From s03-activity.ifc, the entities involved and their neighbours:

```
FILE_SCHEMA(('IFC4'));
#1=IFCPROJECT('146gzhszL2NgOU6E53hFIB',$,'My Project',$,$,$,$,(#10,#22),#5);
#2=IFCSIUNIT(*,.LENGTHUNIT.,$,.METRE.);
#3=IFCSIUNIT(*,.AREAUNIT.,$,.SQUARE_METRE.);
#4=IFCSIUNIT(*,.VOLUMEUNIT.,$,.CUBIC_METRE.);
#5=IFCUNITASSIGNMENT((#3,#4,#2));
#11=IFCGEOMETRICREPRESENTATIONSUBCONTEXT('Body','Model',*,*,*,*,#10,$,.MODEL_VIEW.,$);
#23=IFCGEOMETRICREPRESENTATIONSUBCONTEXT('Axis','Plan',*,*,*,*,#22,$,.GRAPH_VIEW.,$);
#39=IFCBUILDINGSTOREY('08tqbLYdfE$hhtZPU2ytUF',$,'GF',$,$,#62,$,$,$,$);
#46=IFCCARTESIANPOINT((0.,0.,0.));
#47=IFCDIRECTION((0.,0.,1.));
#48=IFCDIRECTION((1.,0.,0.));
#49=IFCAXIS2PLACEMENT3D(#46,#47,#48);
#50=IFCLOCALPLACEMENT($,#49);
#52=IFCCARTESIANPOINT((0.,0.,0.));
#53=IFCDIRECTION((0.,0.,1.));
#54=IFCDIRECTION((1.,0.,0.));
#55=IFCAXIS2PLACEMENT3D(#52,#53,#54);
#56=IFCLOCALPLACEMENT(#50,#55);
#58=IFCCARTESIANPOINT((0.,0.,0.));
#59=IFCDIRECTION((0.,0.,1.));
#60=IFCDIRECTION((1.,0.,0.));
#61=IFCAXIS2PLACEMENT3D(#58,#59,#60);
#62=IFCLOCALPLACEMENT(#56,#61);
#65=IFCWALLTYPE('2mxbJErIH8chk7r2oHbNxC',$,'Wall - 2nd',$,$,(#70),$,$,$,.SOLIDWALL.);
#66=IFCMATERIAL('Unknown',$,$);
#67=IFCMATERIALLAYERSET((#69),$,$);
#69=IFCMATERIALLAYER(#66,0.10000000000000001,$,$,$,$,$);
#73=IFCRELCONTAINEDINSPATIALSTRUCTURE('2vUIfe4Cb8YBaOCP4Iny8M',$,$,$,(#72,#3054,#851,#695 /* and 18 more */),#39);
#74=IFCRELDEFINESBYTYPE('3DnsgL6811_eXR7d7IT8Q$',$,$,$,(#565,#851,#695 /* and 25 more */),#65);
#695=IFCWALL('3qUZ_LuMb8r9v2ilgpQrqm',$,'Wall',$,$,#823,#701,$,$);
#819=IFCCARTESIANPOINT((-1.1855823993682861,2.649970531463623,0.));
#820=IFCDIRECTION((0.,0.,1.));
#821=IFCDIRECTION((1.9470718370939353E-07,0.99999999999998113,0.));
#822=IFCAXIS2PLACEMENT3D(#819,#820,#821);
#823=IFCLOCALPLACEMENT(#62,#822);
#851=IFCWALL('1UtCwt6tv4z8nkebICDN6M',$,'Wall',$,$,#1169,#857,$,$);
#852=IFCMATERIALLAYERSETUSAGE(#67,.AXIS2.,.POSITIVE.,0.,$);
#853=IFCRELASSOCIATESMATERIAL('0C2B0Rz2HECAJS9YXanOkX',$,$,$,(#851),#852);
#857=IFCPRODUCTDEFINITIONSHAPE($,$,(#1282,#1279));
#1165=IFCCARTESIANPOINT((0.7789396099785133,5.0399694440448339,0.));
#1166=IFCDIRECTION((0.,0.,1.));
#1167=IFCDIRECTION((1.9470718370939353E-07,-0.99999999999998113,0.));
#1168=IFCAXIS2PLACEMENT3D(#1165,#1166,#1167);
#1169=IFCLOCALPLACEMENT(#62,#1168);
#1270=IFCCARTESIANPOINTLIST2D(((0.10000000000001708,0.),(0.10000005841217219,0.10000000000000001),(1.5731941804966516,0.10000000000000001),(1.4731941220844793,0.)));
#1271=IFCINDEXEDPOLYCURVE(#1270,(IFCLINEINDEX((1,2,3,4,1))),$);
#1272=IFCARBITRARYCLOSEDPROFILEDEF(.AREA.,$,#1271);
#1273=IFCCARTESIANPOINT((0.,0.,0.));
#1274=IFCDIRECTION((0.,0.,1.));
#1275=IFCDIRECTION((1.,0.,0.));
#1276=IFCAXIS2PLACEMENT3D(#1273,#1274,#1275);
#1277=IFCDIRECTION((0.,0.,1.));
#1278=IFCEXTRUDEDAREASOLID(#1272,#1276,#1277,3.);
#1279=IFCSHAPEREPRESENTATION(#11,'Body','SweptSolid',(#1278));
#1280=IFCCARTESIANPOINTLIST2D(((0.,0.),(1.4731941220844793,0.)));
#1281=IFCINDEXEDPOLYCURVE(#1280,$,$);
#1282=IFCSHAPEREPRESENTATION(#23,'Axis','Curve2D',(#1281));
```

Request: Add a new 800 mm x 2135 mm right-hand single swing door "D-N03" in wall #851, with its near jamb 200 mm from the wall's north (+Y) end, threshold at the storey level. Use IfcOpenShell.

```python
import numpy as np
import ifcopenshell
import ifcopenshell.api.feature
import ifcopenshell.api.geometry
import ifcopenshell.api.root
import ifcopenshell.api.spatial
import ifcopenshell.geom
import ifcopenshell.util.element
import ifcopenshell.util.placement
import ifcopenshell.util.representation
import ifcopenshell.util.shape
import ifcopenshell.util.unit

model = ifcopenshell.open("s03-activity.ifc")
unit_scale = ifcopenshell.util.unit.calculate_unit_scale(model)
settings = ifcopenshell.geom.settings()


def volume(element):
    """Net volume in cubic metres, openings subtracted."""
    shape = ifcopenshell.geom.create_shape(settings, element)
    return ifcopenshell.util.shape.get_volume(shape.geometry)


wall = model.by_guid("1UtCwt6tv4z8nkebICDN6M")
storey = ifcopenshell.util.element.get_container(wall, ifc_class="IfcBuildingStorey")
context = ifcopenshell.util.representation.get_context(model, "Model", "Body", "MODEL_VIEW")
before = volume(wall)

width, height, from_end, sill = 0.8, 2.135, 0.2, 0.0  # metres

# The wall runs along its own X axis, and the end named is its -X end.
wall_shape = ifcopenshell.geom.create_shape(settings, wall)
x, y, z = ifcopenshell.util.shape.get_vertices(wall_shape.geometry).T
start = x.min() + from_end
face, thickness = float(y.min()), float(y.max() - y.min())
wall_matrix = ifcopenshell.util.placement.get_local_placement(wall.ObjectPlacement)
level = ifcopenshell.util.placement.get_local_placement(storey.ObjectPlacement)[2, 3]


def in_wall(x, y):
    """Placement at x, y metres in the wall's axes, at sill height."""
    matrix = wall_matrix.copy()
    matrix[:, 3] = wall_matrix @ np.array([x / unit_scale, y / unit_scale, 0.0, 1.0])
    matrix[2, 3] = level + sill / unit_scale
    return matrix


# Opening: a box that overshoots both wall faces by 50 mm.
opening = ifcopenshell.api.root.create_entity(model, ifc_class="IfcOpeningElement", predefined_type="OPENING")
box = ifcopenshell.api.geometry.add_wall_representation(
    model, context=context, length=width, height=height, thickness=thickness + 0.1
)
ifcopenshell.api.geometry.assign_representation(model, product=opening, representation=box)
ifcopenshell.api.geometry.edit_object_placement(model, product=opening, matrix=in_wall(start, face - 0.05), is_si=False)
ifcopenshell.api.feature.add_feature(model, feature=opening, element=wall)

door = ifcopenshell.api.root.create_entity(model, ifc_class="IfcDoor", name="D-N03", predefined_type="DOOR")
door.OverallWidth, door.OverallHeight = width / unit_scale, height / unit_scale
door.OperationType = "SINGLE_SWING_RIGHT"
body = ifcopenshell.api.geometry.add_door_representation(
    model,
    context=context,
    overall_width=door.OverallWidth,
    overall_height=door.OverallHeight,
    operation_type="SINGLE_SWING_RIGHT",
    lining_properties={"LiningDepth": thickness / unit_scale, "ThresholdDepth": thickness / unit_scale},
)
ifcopenshell.api.geometry.assign_representation(model, product=door, representation=body)
ifcopenshell.api.spatial.assign_container(model, products=[door], relating_structure=storey)
ifcopenshell.api.feature.add_filling(model, opening=opening, element=door)

# The lining spans the wall, so the door starts at the wall face.
ifcopenshell.api.geometry.edit_object_placement(model, product=door, matrix=in_wall(start, face), is_si=False)

after = volume(wall)

print(f"wall volume {before:.3f} -> {after:.3f} m3")

model.write("s03-activity_v2.ifc")
```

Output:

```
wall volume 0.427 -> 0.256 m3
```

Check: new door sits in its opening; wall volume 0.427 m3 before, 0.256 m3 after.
